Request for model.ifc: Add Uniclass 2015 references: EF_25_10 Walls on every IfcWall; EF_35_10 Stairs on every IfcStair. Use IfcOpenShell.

First a look at what the model holds.

```python
import ifcopenshell

model = ifcopenshell.open("model.ifc")
print(model.schema)
print("classifications:", [c.Name for c in model.by_type("IfcClassification")])
for ifc_class in ("IfcDoor", "IfcRoof", "IfcStair", "IfcWall", "IfcWindow"):
    print(ifc_class, len(model.by_type(ifc_class)))
```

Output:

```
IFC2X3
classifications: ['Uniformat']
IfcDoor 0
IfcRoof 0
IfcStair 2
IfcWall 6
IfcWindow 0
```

```python
import ifcopenshell
import ifcopenshell.api.classification

model = ifcopenshell.open("model.ifc")

# IFC2X3 requires Source and Edition and has no link from the project to the system.
system = model.create_entity("IfcClassification", Source="NBS", Edition="2015", Name="Uniclass 2015")

codes = {
    "IfcWall": ("EF_25_10", "Walls"),
    "IfcStair": ("EF_35_10", "Stairs"),
}
for ifc_class, (code, name) in codes.items():
    products = model.by_type(ifc_class)
    ifcopenshell.api.classification.add_reference(
        model, products=products, classification=system, identification=code, name=name
    )
    print(code, len(products))

model.write("model_edited.ifc")
```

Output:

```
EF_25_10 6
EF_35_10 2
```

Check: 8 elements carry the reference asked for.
